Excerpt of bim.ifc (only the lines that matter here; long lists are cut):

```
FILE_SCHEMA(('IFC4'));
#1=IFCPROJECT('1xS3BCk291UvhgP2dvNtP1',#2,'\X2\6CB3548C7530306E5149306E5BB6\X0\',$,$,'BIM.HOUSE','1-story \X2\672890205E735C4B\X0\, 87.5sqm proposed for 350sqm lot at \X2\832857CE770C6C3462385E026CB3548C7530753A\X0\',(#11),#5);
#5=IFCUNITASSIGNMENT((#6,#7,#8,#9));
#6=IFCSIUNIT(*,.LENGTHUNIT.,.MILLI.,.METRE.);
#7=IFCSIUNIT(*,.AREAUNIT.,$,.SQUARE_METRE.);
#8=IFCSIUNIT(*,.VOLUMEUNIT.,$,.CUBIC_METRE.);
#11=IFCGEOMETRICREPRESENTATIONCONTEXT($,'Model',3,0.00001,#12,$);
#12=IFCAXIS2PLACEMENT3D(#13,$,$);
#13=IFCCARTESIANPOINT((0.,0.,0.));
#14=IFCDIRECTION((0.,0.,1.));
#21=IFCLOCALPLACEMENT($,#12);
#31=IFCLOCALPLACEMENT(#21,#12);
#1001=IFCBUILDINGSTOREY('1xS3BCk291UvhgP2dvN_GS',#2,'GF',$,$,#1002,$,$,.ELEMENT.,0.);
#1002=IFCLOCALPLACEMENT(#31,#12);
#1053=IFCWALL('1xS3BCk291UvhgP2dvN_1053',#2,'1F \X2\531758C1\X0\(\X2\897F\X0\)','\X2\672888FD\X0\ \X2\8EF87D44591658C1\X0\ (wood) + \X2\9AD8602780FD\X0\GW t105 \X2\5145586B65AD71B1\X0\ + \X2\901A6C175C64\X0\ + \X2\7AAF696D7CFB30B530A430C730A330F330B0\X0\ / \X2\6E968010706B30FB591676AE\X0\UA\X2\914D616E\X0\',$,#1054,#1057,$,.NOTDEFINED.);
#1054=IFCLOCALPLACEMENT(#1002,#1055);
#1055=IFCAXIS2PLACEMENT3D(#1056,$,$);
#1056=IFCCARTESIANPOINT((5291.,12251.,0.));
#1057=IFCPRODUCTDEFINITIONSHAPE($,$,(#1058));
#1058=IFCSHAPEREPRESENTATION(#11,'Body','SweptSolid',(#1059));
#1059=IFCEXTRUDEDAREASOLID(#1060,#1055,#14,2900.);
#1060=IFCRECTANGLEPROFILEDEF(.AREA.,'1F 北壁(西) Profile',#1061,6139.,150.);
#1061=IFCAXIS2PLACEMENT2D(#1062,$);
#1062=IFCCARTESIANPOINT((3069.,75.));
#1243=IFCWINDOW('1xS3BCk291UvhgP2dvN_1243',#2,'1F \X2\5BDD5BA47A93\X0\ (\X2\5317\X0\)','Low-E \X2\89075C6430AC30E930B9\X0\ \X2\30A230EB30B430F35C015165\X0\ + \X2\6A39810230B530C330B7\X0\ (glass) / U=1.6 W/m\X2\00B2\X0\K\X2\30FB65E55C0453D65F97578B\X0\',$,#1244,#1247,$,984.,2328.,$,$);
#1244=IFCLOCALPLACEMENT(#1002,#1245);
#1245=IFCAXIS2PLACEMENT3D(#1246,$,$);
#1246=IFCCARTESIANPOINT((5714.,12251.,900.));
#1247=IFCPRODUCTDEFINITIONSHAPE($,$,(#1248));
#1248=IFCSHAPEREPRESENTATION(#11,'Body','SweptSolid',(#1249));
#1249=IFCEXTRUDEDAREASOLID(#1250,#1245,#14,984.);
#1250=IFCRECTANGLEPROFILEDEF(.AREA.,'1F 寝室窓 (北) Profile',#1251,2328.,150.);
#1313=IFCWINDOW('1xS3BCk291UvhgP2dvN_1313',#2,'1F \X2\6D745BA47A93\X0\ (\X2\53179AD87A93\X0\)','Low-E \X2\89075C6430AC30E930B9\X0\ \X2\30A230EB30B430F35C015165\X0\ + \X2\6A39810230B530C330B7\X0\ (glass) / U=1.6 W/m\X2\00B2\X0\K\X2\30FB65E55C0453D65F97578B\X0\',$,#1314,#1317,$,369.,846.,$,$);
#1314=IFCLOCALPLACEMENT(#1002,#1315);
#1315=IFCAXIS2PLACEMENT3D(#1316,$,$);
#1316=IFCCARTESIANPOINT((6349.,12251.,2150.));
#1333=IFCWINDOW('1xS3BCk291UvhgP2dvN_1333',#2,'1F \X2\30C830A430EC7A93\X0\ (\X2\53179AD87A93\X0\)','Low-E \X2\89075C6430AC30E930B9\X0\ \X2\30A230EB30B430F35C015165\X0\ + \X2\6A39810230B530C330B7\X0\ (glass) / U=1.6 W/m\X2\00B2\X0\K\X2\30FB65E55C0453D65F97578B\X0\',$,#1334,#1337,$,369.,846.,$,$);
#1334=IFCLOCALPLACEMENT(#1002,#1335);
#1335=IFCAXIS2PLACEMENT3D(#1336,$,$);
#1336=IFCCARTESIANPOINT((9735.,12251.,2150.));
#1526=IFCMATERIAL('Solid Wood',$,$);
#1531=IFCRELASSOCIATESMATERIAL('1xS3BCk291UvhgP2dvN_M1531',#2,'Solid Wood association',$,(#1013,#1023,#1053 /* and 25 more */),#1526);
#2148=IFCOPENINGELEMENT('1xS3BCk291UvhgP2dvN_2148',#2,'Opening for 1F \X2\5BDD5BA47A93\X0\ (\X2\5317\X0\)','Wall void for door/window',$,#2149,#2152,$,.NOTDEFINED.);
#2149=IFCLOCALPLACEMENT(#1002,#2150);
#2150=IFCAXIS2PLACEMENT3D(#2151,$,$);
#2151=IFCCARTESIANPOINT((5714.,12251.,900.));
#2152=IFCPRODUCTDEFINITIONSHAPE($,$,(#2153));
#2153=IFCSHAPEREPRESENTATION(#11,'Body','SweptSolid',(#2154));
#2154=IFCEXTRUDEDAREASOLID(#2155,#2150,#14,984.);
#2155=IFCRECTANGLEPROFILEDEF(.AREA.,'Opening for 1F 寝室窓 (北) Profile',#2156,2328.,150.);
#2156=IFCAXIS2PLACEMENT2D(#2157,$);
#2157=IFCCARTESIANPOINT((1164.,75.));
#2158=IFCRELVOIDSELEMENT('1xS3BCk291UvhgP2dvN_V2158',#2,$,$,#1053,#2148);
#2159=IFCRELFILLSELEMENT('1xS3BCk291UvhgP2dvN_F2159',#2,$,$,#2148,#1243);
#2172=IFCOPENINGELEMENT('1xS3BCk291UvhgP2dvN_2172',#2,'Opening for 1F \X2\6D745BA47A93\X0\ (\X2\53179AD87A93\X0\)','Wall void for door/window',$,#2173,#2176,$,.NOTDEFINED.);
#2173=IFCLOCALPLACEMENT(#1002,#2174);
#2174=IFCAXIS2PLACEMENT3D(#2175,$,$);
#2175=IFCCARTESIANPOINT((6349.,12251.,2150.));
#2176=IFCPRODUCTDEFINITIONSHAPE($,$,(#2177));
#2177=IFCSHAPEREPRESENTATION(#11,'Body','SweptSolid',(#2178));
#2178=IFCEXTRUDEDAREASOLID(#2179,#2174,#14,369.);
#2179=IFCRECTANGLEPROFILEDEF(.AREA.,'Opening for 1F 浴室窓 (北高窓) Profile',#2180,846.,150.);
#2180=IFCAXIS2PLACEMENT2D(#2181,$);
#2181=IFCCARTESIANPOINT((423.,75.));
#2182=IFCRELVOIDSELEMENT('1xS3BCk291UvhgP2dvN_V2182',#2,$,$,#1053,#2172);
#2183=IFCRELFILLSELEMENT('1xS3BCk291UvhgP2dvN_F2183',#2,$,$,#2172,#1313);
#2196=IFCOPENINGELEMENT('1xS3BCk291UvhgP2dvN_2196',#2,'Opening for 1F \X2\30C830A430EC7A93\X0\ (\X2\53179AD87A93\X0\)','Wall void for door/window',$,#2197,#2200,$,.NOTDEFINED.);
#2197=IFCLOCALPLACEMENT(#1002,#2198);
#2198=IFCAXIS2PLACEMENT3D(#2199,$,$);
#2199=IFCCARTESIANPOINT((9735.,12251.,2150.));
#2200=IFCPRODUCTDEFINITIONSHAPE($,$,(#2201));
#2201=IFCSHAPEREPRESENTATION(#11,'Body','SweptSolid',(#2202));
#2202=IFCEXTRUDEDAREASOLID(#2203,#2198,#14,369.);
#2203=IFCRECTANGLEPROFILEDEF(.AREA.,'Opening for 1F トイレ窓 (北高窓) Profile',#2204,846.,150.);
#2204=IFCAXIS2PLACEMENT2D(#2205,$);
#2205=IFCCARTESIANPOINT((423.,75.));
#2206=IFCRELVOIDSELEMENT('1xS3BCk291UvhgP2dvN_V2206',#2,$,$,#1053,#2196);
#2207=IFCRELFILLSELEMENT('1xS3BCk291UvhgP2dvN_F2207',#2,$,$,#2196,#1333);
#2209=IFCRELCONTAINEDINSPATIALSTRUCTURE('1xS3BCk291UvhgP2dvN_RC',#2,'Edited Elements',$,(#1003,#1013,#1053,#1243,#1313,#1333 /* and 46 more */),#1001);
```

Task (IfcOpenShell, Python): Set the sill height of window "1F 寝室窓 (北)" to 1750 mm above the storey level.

```python
import numpy as np
import ifcopenshell
import ifcopenshell.api.geometry
import ifcopenshell.geom
import ifcopenshell.util.element
import ifcopenshell.util.placement
import ifcopenshell.util.shape
import ifcopenshell.util.unit

model = ifcopenshell.open("bim.ifc")
unit_scale = ifcopenshell.util.unit.calculate_unit_scale(model)

window = model.by_id(1243)
opening = window.FillsVoids[0].RelatingOpeningElement
storey = ifcopenshell.util.element.get_container(window, ifc_class="IfcBuildingStorey")
level = ifcopenshell.util.placement.get_local_placement(storey.ObjectPlacement)[2, 3]

# The opening's origin need not be at the sill, so measure its lowest point.
shape = ifcopenshell.geom.create_shape(ifcopenshell.geom.settings(), opening)
bottom = ifcopenshell.util.shape.get_shape_bottom_elevation(shape, shape.geometry) / unit_scale
dz = level + 1.75 / unit_scale - bottom

shift = np.array([0.0, 0.0, dz])
# The window is not placed relative to its opening, so move both.
for product in (opening, window):
    matrix = ifcopenshell.util.placement.get_local_placement(product.ObjectPlacement)
    matrix[:3, 3] += shift
    ifcopenshell.api.geometry.edit_object_placement(model, product=product, matrix=matrix, is_si=False)

print(f"moved by {dz * unit_scale:+.3f} m")

model.write("bim_updated.ifc")
```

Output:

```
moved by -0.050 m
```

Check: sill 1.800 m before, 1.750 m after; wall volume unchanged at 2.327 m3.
